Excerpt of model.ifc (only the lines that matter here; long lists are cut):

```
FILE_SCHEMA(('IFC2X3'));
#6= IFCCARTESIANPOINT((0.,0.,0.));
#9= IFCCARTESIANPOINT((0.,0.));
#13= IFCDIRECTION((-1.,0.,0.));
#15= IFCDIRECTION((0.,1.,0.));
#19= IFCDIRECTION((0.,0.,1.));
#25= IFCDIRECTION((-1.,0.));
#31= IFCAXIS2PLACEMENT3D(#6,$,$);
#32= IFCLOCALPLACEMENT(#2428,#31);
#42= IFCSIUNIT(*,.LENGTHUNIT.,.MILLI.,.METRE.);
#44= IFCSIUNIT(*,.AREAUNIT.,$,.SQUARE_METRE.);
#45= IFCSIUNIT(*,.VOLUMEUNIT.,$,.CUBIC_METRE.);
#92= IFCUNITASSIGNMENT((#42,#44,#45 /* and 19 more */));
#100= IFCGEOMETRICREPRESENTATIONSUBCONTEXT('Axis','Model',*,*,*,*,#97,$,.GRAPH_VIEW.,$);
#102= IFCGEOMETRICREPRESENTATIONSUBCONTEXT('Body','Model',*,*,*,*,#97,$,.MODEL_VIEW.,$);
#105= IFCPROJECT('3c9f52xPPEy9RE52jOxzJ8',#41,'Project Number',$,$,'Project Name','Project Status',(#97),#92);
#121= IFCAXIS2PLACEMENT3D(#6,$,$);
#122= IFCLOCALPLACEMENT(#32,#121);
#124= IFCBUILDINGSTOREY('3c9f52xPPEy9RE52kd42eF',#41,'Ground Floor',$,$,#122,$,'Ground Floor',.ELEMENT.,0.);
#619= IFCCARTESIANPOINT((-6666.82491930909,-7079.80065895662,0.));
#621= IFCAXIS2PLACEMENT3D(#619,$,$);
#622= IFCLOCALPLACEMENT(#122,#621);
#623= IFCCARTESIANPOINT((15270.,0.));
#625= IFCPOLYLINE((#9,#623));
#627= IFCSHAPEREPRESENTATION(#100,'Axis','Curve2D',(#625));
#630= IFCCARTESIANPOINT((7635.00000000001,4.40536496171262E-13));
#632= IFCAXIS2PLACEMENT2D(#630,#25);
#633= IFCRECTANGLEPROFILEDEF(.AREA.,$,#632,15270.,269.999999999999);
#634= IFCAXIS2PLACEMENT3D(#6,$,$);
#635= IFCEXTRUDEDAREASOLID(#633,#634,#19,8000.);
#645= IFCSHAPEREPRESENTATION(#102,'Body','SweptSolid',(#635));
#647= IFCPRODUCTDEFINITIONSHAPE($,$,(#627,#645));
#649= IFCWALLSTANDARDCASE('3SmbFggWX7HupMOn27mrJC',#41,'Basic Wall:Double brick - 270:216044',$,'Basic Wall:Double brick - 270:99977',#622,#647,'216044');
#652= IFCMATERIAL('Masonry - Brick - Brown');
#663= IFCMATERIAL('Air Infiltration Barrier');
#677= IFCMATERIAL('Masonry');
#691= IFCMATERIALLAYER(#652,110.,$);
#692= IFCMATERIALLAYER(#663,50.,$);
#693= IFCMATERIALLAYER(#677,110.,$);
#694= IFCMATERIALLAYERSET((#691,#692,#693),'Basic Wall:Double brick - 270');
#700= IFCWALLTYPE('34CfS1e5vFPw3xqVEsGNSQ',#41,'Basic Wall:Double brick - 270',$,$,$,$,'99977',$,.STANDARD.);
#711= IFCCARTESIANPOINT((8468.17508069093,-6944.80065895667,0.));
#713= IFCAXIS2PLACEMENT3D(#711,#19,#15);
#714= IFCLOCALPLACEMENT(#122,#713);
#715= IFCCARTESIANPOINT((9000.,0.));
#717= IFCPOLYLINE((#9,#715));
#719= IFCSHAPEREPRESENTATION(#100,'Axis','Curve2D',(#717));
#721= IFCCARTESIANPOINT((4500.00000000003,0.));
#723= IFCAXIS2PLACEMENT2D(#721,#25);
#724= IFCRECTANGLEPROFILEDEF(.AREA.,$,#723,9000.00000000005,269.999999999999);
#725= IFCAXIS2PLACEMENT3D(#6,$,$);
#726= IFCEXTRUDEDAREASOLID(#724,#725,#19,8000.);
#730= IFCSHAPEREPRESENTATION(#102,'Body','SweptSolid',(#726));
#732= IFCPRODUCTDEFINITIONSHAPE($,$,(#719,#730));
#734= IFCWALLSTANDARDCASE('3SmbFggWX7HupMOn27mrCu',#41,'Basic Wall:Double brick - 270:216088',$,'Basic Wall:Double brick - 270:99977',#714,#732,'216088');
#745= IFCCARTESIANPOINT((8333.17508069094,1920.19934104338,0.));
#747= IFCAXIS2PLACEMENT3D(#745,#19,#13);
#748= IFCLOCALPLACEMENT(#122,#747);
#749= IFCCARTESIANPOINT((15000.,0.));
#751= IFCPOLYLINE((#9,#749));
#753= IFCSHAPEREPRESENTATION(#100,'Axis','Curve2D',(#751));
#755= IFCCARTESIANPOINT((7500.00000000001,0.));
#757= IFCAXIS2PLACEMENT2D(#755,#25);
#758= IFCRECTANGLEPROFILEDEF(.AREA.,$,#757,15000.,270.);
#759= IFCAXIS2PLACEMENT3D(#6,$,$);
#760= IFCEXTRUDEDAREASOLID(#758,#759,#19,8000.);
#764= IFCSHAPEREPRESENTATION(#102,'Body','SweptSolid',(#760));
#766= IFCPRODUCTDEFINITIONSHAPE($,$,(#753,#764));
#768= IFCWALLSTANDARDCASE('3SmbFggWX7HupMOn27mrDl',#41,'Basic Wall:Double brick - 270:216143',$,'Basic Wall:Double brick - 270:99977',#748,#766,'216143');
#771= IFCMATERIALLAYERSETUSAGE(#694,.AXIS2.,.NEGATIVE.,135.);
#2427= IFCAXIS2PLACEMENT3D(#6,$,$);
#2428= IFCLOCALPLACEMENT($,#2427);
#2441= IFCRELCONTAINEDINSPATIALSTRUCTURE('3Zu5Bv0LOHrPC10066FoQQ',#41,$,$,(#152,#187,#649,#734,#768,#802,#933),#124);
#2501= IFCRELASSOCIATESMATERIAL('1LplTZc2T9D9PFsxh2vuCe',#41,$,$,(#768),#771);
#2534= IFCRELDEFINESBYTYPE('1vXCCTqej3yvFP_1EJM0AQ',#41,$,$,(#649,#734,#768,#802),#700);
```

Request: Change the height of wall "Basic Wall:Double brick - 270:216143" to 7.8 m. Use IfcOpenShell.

```python
import ifcopenshell
import ifcopenshell.geom
import ifcopenshell.util.representation
import ifcopenshell.util.shape
import ifcopenshell.util.unit

model = ifcopenshell.open("model.ifc")
unit_scale = ifcopenshell.util.unit.calculate_unit_scale(model)
settings = ifcopenshell.geom.settings()


def volume(element):
    """Net volume in cubic metres, openings subtracted."""
    shape = ifcopenshell.geom.create_shape(settings, element)
    return ifcopenshell.util.shape.get_volume(shape.geometry)


wall = model.by_guid("3SmbFggWX7HupMOn27mrDl")
before = volume(wall)

body = ifcopenshell.util.representation.get_representation(wall, "Model", "Body")
solid = body.Items[0]
old_height = solid.Depth
solid.Depth = 7.8 / unit_scale
after = volume(wall)

print(f"height {old_height:g} -> {solid.Depth:g}, volume {before:.3f} -> {after:.3f} m3")

model.write("model_rev.ifc")
```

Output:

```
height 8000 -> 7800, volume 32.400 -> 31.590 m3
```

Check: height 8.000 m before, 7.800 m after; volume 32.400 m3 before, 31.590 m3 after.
